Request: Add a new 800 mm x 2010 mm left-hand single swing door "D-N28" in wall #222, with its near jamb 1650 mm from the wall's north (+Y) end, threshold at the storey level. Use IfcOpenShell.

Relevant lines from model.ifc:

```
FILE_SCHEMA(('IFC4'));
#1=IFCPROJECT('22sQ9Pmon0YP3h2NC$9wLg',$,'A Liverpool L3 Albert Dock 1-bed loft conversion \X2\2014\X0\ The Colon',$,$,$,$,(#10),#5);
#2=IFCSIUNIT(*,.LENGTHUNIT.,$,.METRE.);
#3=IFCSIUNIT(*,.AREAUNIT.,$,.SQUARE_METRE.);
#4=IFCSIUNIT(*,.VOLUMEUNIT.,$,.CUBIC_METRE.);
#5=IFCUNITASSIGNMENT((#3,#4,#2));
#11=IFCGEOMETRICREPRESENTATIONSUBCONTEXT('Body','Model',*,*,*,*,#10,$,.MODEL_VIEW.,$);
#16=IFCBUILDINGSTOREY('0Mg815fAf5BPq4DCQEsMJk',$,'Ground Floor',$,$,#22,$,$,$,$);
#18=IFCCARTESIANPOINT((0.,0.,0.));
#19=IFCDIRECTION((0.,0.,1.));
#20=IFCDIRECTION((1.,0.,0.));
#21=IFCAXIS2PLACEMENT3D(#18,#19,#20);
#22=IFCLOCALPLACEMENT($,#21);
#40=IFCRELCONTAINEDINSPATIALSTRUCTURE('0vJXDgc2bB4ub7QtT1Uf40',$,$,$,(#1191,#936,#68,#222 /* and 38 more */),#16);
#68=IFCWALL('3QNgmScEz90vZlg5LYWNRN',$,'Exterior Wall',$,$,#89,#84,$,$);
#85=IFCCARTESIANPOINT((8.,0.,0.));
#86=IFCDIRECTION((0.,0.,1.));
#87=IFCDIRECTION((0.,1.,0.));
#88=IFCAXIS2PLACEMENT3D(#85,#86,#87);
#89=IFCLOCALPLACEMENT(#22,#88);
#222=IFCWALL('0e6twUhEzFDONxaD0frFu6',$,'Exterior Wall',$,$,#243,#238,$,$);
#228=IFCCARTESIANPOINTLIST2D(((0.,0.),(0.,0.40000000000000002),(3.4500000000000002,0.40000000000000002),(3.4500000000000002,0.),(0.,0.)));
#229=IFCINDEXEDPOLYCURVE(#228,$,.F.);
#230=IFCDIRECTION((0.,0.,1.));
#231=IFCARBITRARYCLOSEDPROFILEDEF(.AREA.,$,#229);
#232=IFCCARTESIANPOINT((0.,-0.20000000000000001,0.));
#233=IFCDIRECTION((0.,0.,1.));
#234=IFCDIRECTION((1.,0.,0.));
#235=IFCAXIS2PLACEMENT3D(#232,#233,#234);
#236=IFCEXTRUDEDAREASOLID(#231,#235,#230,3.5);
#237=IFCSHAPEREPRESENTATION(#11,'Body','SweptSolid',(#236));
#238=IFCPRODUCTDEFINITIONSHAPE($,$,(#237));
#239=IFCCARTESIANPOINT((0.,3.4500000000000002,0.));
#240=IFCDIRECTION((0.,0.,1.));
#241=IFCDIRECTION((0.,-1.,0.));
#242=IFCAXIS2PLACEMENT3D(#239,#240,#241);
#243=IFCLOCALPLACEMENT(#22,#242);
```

```python
import numpy as np
import ifcopenshell
import ifcopenshell.api.feature
import ifcopenshell.api.geometry
import ifcopenshell.api.root
import ifcopenshell.api.spatial
import ifcopenshell.geom
import ifcopenshell.util.element
import ifcopenshell.util.placement
import ifcopenshell.util.representation
import ifcopenshell.util.shape
import ifcopenshell.util.unit

model = ifcopenshell.open("model.ifc")
unit_scale = ifcopenshell.util.unit.calculate_unit_scale(model)
settings = ifcopenshell.geom.settings()


def volume(element):
    """Net volume in cubic metres, openings subtracted."""
    shape = ifcopenshell.geom.create_shape(settings, element)
    return ifcopenshell.util.shape.get_volume(shape.geometry)


wall = model.by_id(222)
storey = ifcopenshell.util.element.get_container(wall, ifc_class="IfcBuildingStorey")
context = ifcopenshell.util.representation.get_context(model, "Model", "Body", "MODEL_VIEW")
before = volume(wall)

width, height, from_end, sill = 0.8, 2.01, 1.65, 0.0  # metres

# The wall runs along its own X axis, and the end named is its -X end.
wall_shape = ifcopenshell.geom.create_shape(settings, wall)
x, y, z = ifcopenshell.util.shape.get_vertices(wall_shape.geometry).T
start = x.min() + from_end
face, thickness = float(y.min()), float(y.max() - y.min())
wall_matrix = ifcopenshell.util.placement.get_local_placement(wall.ObjectPlacement)
level = ifcopenshell.util.placement.get_local_placement(storey.ObjectPlacement)[2, 3]


def in_wall(x, y):
    """Placement at x, y metres in the wall's axes, at sill height."""
    matrix = wall_matrix.copy()
    matrix[:, 3] = wall_matrix @ np.array([x / unit_scale, y / unit_scale, 0.0, 1.0])
    matrix[2, 3] = level + sill / unit_scale
    return matrix


# Opening: a box that overshoots both wall faces by 50 mm.
opening = ifcopenshell.api.root.create_entity(model, ifc_class="IfcOpeningElement", predefined_type="OPENING")
box = ifcopenshell.api.geometry.add_wall_representation(
    model, context=context, length=width, height=height, thickness=thickness + 0.1
)
ifcopenshell.api.geometry.assign_representation(model, product=opening, representation=box)
ifcopenshell.api.geometry.edit_object_placement(model, product=opening, matrix=in_wall(start, face - 0.05), is_si=False)
ifcopenshell.api.feature.add_feature(model, feature=opening, element=wall)

door = ifcopenshell.api.root.create_entity(model, ifc_class="IfcDoor", name="D-N28", predefined_type="DOOR")
door.OverallWidth, door.OverallHeight = width / unit_scale, height / unit_scale
door.OperationType = "SINGLE_SWING_LEFT"
body = ifcopenshell.api.geometry.add_door_representation(
    model,
    context=context,
    overall_width=door.OverallWidth,
    overall_height=door.OverallHeight,
    operation_type="SINGLE_SWING_LEFT",
    lining_properties={"LiningDepth": thickness / unit_scale, "ThresholdDepth": thickness / unit_scale},
)
ifcopenshell.api.geometry.assign_representation(model, product=door, representation=body)
ifcopenshell.api.spatial.assign_container(model, products=[door], relating_structure=storey)
ifcopenshell.api.feature.add_filling(model, opening=opening, element=door)

# The lining spans the wall, so the door starts at the wall face.
ifcopenshell.api.geometry.edit_object_placement(model, product=door, matrix=in_wall(start, face), is_si=False)

after = volume(wall)

print(f"wall volume {before:.3f} -> {after:.3f} m3")

model.write("model_rev.ifc")
```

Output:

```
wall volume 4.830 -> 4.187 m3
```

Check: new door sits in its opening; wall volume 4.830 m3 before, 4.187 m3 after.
